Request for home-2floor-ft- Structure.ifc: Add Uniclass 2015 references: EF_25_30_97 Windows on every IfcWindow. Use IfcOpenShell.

First a look at what the model holds.

```python
import ifcopenshell

model = ifcopenshell.open("home-2floor-ft- Structure.ifc")
print(model.schema)
print("classifications:", [c.Name for c in model.by_type("IfcClassification")])
for ifc_class in ("IfcDoor", "IfcRoof", "IfcStair", "IfcWall", "IfcWindow"):
    print(ifc_class, len(model.by_type(ifc_class)))
```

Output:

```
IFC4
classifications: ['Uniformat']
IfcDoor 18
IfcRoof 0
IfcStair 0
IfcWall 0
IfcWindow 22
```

```python
import ifcopenshell
import ifcopenshell.api.classification

model = ifcopenshell.open("home-2floor-ft- Structure.ifc")

system = ifcopenshell.api.classification.add_classification(model, classification="Uniclass 2015")

codes = {
    "IfcWindow": ("EF_25_30_97", "Windows"),
}
for ifc_class, (code, name) in codes.items():
    products = model.by_type(ifc_class)
    ifcopenshell.api.classification.add_reference(
        model, products=products, classification=system, identification=code, name=name
    )
    print(code, len(products))

model.write("home-2floor-ft- Structure-out.ifc")
```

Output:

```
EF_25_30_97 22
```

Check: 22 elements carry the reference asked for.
